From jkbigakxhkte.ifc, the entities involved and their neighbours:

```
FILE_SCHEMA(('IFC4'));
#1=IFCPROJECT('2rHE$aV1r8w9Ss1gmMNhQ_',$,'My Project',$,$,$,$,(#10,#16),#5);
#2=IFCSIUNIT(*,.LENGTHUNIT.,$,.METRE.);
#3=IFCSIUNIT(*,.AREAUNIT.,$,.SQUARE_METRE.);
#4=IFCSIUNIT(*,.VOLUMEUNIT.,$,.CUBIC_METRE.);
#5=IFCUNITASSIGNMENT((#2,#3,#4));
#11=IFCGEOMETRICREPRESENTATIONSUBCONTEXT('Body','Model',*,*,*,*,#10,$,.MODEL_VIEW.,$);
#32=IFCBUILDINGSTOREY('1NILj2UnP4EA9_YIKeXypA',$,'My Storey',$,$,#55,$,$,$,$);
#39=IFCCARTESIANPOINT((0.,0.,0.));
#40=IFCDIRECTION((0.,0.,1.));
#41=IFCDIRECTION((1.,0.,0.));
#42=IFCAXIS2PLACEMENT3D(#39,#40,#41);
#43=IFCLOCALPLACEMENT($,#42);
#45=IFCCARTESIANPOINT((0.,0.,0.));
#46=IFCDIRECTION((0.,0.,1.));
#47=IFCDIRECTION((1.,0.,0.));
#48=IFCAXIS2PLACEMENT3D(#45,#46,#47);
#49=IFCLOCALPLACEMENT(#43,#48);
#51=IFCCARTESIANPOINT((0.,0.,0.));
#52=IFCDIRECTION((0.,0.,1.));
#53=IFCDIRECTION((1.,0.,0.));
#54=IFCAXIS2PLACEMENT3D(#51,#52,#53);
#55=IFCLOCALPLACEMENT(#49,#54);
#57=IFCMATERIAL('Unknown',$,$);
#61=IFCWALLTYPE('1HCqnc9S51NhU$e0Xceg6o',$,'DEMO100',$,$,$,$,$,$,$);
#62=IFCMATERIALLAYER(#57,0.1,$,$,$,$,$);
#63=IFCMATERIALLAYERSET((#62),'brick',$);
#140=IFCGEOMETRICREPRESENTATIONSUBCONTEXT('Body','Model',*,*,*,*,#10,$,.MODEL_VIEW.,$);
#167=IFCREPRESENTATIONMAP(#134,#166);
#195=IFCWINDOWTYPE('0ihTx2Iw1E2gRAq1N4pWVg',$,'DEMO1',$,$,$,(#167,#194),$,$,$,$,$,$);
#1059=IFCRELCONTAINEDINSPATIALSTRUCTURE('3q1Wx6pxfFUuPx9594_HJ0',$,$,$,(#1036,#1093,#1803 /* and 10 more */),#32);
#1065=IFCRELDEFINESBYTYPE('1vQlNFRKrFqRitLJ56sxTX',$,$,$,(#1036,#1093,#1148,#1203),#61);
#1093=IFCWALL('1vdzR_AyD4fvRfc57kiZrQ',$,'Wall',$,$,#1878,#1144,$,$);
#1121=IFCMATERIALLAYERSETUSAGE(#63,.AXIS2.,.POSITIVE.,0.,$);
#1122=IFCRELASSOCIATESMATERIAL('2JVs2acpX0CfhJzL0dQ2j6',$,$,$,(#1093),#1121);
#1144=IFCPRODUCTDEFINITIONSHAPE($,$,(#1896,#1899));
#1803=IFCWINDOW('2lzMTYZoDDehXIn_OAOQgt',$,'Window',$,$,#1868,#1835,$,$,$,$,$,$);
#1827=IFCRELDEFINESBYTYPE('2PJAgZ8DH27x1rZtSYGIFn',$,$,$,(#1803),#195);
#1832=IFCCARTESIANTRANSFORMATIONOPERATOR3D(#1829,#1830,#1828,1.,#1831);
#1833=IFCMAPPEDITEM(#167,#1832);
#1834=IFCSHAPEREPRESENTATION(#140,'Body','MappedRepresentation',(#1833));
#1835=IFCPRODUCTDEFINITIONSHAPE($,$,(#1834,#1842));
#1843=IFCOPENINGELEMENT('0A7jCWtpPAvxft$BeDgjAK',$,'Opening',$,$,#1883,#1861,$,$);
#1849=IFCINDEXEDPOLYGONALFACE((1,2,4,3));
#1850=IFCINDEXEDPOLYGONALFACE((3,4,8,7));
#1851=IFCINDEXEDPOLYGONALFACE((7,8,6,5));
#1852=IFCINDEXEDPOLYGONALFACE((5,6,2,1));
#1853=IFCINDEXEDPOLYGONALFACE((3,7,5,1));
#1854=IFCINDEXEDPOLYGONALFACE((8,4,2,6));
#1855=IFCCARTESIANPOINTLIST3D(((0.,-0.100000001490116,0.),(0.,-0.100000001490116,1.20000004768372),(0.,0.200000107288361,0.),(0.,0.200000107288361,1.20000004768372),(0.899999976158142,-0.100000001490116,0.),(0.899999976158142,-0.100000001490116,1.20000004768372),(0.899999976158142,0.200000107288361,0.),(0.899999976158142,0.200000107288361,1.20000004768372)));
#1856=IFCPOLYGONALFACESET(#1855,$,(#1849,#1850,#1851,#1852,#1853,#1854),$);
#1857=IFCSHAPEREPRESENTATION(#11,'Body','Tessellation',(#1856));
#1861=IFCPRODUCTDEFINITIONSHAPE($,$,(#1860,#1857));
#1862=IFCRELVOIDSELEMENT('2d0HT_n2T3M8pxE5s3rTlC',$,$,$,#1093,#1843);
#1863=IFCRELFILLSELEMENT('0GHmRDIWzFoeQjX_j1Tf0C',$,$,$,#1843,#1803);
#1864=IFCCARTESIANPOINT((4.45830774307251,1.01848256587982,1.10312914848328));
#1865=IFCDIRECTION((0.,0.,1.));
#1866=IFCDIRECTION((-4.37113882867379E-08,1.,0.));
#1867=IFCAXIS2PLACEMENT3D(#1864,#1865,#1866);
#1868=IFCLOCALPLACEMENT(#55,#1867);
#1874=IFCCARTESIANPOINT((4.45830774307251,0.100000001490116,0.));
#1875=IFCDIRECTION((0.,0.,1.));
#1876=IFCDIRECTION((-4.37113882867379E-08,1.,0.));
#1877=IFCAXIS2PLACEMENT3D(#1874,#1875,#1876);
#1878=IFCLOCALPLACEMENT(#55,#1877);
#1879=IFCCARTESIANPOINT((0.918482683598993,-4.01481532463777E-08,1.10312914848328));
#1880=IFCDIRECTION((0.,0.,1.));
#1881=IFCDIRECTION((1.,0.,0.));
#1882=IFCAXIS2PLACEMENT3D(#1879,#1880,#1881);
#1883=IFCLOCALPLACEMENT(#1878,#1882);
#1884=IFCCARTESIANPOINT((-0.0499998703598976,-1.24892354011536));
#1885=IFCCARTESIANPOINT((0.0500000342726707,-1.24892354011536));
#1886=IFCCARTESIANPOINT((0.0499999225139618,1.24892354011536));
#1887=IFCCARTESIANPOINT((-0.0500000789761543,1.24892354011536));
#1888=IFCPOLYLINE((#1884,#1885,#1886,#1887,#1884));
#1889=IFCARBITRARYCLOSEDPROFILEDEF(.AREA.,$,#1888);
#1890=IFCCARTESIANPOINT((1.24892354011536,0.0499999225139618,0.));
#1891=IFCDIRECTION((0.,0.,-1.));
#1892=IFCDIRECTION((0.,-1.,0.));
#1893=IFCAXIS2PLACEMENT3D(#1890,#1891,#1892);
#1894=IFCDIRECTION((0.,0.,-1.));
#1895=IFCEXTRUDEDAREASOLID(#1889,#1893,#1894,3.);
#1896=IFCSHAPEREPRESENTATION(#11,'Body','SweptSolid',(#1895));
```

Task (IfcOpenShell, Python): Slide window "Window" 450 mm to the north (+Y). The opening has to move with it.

```python
import ifcopenshell
import ifcopenshell.api.geometry
import ifcopenshell.util.placement
import ifcopenshell.util.unit

model = ifcopenshell.open("jkbigakxhkte.ifc")
unit_scale = ifcopenshell.util.unit.calculate_unit_scale(model)

window = model.by_guid("2lzMTYZoDDehXIn_OAOQgt")
opening = window.FillsVoids[0].RelatingOpeningElement
wall = opening.VoidsElements[0].RelatingBuildingElement

wall_matrix = ifcopenshell.util.placement.get_local_placement(wall.ObjectPlacement)
shift = wall_matrix[:3, 0] * 0.45 / unit_scale
before = ifcopenshell.util.placement.get_local_placement(window.ObjectPlacement)[:3, 3].copy()

# The window is not placed relative to its opening, so move both.
for product in (opening, window):
    matrix = ifcopenshell.util.placement.get_local_placement(product.ObjectPlacement)
    matrix[:3, 3] += shift
    ifcopenshell.api.geometry.edit_object_placement(model, product=product, matrix=matrix, is_si=False)

after = ifcopenshell.util.placement.get_local_placement(window.ObjectPlacement)[:3, 3]
print("window moved by", (after - before).round(3) + 0.0)

model.write("jkbigakxhkte_rev.ifc")
```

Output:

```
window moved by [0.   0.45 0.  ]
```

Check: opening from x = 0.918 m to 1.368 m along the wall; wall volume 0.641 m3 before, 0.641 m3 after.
